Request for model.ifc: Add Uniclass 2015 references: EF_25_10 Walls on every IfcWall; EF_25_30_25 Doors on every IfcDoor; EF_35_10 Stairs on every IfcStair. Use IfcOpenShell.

First a look at what the model holds.

```python
import ifcopenshell

model = ifcopenshell.open("model.ifc")
print(model.schema)
print("classifications:", [c.Name for c in model.by_type("IfcClassification")])
for ifc_class in ("IfcDoor", "IfcRoof", "IfcStair", "IfcWall", "IfcWindow"):
    print(ifc_class, len(model.by_type(ifc_class)))
```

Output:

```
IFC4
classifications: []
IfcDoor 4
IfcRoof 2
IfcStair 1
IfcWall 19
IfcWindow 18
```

```python
import ifcopenshell
import ifcopenshell.api.classification

model = ifcopenshell.open("model.ifc")

system = ifcopenshell.api.classification.add_classification(model, classification="Uniclass 2015")

codes = {
    "IfcWall": ("EF_25_10", "Walls"),
    "IfcDoor": ("EF_25_30_25", "Doors"),
    "IfcStair": ("EF_35_10", "Stairs"),
}
for ifc_class, (code, name) in codes.items():
    products = model.by_type(ifc_class)
    ifcopenshell.api.classification.add_reference(
        model, products=products, classification=system, identification=code, name=name
    )
    print(code, len(products))

model.write("model-out.ifc")
```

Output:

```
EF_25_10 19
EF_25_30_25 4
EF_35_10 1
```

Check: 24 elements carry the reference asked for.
